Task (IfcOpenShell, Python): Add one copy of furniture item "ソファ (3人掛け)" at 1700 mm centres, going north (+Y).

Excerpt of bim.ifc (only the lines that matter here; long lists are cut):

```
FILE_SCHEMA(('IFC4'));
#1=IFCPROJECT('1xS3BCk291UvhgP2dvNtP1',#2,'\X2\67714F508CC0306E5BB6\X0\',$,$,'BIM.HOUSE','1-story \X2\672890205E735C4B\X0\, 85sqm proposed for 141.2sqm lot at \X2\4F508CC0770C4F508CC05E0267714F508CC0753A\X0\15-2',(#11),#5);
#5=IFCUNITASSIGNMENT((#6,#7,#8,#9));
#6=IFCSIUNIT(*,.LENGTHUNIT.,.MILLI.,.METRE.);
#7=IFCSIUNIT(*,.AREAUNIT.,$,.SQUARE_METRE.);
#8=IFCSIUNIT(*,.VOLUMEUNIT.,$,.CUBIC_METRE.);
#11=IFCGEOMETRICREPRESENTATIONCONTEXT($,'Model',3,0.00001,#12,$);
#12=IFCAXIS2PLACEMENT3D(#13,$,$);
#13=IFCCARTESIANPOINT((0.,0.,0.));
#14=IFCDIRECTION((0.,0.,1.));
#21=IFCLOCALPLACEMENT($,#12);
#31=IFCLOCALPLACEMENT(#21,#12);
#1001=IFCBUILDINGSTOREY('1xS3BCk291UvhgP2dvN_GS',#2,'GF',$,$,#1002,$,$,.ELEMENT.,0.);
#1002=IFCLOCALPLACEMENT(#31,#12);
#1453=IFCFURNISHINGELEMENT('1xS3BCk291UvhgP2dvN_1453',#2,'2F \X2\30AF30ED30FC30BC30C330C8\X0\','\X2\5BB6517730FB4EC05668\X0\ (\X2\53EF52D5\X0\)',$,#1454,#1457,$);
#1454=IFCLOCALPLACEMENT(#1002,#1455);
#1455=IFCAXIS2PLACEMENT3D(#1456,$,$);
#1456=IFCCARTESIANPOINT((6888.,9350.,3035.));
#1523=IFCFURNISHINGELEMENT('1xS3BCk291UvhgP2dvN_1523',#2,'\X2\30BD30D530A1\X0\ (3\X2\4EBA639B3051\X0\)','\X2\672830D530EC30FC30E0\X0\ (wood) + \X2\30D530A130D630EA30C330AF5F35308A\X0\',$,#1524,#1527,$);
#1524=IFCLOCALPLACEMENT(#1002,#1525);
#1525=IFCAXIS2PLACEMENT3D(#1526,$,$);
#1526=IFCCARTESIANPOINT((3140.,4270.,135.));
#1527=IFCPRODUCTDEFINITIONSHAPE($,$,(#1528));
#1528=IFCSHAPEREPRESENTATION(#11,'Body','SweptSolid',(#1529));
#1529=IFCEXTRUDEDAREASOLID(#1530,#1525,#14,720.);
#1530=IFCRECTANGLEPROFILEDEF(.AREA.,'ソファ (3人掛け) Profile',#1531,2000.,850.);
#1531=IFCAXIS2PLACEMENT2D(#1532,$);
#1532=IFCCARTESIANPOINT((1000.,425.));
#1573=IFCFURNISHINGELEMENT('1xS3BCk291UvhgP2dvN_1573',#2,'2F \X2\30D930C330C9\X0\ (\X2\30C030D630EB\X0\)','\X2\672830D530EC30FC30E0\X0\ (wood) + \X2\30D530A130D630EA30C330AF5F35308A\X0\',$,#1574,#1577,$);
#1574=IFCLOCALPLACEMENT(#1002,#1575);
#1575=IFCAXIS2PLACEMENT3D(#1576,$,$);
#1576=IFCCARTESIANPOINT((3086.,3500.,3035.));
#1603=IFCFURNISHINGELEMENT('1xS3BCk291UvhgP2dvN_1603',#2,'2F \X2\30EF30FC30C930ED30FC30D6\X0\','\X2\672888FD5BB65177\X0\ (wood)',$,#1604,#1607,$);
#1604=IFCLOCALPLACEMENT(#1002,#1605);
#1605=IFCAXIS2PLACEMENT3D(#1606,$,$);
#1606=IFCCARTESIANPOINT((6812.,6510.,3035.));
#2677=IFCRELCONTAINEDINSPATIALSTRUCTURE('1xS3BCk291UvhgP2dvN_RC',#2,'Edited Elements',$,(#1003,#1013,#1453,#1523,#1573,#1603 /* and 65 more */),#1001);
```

```python
import numpy as np
import ifcopenshell
import ifcopenshell.api.geometry
import ifcopenshell.api.root
import ifcopenshell.util.element
import ifcopenshell.util.placement

model = ifcopenshell.open("bim.ifc")


def reuse_history(source, copy):
    """copy_class also copies each property set's owner history, people and application; keep the originals."""
    for rel in copy.IsDefinedBy:
        if rel.is_a("IfcRelDefinesByProperties") and (history := rel.RelatingPropertyDefinition.OwnerHistory):
            rel.RelatingPropertyDefinition.OwnerHistory = source.OwnerHistory
            ifcopenshell.util.element.remove_deep2(model, history)


source = model.by_guid("1xS3BCk291UvhgP2dvN_1523")
base = ifcopenshell.util.placement.get_local_placement(source.ObjectPlacement)
step = np.array([0.0, 1.0, 0.0]) * 1700.0

for i in range(1, 2):
    copy = ifcopenshell.api.root.copy_class(model, product=source)
    copy.Representation = ifcopenshell.util.element.copy_deep(
        model, source.Representation, exclude=["IfcGeometricRepresentationContext", "IfcRepresentationMap"]
    )
    reuse_history(source, copy)
    matrix = base.copy()
    matrix[:3, 3] += i * step
    print("added at", matrix[:3, 3].round(3) + 0.0)
    ifcopenshell.api.geometry.edit_object_placement(model, product=copy, matrix=matrix, is_si=False)

model.write("bim_v2.ifc")
```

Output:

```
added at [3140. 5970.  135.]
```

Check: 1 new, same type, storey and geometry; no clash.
